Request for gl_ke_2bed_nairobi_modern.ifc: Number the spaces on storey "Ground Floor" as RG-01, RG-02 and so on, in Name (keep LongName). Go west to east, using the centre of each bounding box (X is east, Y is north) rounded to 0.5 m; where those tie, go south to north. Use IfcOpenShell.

First a look at what the model holds.

```python
import ifcopenshell
import ifcopenshell.util.element
import ifcopenshell.util.placement

model = ifcopenshell.open("gl_ke_2bed_nairobi_modern.ifc")
print(model.schema)
storey = next(s for s in model.by_type("IfcBuildingStorey") if s.Name == "Ground Floor")
spaces = [e for e in ifcopenshell.util.element.get_decomposition(storey) if e.is_a("IfcSpace")]
for e in sorted(spaces, key=lambda e: e.id()):
    origin = ifcopenshell.util.placement.get_local_placement(e.ObjectPlacement)[:3, 3]
    print(e.id(), e.Name, e.LongName, origin.round(2) + 0.0, sep=" | ")
```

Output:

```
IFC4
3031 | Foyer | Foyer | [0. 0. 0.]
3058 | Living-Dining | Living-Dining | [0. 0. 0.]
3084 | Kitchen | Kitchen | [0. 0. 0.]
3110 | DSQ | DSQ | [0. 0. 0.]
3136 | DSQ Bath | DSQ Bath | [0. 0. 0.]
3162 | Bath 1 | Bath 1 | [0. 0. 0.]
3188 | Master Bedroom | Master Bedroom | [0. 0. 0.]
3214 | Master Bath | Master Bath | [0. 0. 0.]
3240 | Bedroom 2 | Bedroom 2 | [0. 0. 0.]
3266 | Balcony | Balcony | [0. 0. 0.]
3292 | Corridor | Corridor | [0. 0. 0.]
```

```python
import ifcopenshell
import ifcopenshell.geom
import ifcopenshell.util.element
import ifcopenshell.util.shape

model = ifcopenshell.open("gl_ke_2bed_nairobi_modern.ifc")
settings = ifcopenshell.geom.settings()
settings.set("use-world-coords", True)


def centre(element):
    shape = ifcopenshell.geom.create_shape(settings, element)
    return ifcopenshell.util.shape.get_bbox_centroid(shape.geometry)


storey = next(s for s in model.by_type("IfcBuildingStorey") if s.Name == "Ground Floor")
spaces = [e for e in ifcopenshell.util.element.get_decomposition(storey) if e.is_a("IfcSpace")]

# Insertion points can sit at a corner or the storey origin, so sort by the geometry (in metres).
centres = {e: centre(e) for e in spaces}
spaces.sort(key=lambda e: (round(centres[e][0] / 0.5), centres[e][1]))

for i, e in enumerate(spaces, start=1):
    number = f"RG-{i:02d}"
    e.Name = number
    print(e.id(), number)

model.write("gl_ke_2bed_nairobi_modern_updated.ifc")
```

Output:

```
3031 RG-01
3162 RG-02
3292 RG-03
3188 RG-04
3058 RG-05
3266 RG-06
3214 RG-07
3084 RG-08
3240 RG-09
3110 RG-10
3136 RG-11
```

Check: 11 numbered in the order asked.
